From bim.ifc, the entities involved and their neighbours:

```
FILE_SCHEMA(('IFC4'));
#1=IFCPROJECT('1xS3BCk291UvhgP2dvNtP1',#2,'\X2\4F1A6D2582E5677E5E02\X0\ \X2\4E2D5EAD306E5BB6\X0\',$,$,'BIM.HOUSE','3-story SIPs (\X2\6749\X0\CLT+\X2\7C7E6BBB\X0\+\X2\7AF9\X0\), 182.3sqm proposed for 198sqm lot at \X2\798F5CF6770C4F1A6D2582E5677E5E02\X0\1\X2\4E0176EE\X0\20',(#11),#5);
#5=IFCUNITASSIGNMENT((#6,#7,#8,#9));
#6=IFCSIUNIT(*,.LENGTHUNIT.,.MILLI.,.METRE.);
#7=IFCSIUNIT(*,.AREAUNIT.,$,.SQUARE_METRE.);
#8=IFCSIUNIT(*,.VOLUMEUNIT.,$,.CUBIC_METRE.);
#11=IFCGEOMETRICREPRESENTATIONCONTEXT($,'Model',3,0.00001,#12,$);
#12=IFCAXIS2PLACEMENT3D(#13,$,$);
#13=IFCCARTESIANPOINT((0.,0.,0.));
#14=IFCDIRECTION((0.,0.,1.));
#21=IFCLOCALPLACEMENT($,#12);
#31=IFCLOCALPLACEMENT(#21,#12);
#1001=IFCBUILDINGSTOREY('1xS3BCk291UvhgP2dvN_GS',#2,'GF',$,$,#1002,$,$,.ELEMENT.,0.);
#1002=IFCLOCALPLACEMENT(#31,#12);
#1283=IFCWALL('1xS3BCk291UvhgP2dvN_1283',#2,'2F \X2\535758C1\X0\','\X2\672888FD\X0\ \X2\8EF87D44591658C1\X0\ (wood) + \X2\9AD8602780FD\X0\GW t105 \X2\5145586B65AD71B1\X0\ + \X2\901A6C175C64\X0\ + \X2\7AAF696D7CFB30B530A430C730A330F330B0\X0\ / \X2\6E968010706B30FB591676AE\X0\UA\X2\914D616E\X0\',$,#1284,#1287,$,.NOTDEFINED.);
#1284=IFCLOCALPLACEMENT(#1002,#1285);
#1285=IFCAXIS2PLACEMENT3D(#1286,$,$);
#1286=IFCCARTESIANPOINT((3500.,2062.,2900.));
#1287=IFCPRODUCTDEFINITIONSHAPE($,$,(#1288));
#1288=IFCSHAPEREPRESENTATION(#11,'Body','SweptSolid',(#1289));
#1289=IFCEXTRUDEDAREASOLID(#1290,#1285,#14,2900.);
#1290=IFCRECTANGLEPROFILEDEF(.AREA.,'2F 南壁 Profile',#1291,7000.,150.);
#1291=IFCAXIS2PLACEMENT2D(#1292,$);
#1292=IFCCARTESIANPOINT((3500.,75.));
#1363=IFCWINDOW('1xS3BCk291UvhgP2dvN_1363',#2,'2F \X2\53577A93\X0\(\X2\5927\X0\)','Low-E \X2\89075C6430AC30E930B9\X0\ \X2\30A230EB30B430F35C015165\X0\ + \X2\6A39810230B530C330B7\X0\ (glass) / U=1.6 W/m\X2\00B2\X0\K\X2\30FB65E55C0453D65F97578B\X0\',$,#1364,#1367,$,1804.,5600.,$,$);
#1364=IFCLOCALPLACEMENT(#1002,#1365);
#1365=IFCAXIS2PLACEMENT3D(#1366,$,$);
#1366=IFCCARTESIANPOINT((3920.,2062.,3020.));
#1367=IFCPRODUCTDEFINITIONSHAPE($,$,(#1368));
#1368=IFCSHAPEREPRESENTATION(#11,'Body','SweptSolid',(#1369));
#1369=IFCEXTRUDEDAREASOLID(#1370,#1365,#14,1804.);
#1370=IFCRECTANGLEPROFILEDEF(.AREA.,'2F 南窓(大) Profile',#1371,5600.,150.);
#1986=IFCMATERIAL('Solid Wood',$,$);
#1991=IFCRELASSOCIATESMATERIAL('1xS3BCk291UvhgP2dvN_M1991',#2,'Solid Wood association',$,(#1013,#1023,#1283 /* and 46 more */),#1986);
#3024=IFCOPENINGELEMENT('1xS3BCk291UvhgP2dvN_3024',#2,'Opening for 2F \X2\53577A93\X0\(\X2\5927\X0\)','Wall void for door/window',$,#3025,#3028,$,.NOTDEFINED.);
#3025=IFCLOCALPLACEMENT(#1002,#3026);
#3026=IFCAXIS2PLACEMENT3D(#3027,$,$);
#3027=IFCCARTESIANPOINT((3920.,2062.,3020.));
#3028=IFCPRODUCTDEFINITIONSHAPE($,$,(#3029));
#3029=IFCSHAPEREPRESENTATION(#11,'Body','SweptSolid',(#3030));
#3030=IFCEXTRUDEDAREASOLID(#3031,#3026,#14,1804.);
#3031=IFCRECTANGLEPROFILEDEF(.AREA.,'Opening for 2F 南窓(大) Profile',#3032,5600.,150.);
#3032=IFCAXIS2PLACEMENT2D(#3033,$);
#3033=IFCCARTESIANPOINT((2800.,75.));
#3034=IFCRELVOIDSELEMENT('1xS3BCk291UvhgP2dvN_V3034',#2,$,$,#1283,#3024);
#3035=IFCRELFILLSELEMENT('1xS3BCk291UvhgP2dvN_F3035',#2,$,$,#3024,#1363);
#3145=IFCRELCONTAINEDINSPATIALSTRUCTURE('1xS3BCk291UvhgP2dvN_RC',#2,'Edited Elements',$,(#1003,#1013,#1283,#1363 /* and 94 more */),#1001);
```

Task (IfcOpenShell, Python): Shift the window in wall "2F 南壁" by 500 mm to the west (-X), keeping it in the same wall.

```python
import ifcopenshell
import ifcopenshell.api.geometry
import ifcopenshell.util.placement

model = ifcopenshell.open("bim.ifc")

window = model.by_id(1363)
opening = window.FillsVoids[0].RelatingOpeningElement
wall = opening.VoidsElements[0].RelatingBuildingElement

wall_matrix = ifcopenshell.util.placement.get_local_placement(wall.ObjectPlacement)
shift = wall_matrix[:3, 0] * -500.0
before = ifcopenshell.util.placement.get_local_placement(window.ObjectPlacement)[:3, 3].copy()

# The window is not placed relative to its opening, so move both.
for product in (opening, window):
    matrix = ifcopenshell.util.placement.get_local_placement(product.ObjectPlacement)
    matrix[:3, 3] += shift
    ifcopenshell.api.geometry.edit_object_placement(model, product=product, matrix=matrix, is_si=False)

after = ifcopenshell.util.placement.get_local_placement(window.ObjectPlacement)[:3, 3]
print("window moved by", (after - before).round(3) + 0.0)

model.write("bim_rev.ifc")
```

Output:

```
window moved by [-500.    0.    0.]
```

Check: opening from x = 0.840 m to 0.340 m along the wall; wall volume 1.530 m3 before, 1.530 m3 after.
